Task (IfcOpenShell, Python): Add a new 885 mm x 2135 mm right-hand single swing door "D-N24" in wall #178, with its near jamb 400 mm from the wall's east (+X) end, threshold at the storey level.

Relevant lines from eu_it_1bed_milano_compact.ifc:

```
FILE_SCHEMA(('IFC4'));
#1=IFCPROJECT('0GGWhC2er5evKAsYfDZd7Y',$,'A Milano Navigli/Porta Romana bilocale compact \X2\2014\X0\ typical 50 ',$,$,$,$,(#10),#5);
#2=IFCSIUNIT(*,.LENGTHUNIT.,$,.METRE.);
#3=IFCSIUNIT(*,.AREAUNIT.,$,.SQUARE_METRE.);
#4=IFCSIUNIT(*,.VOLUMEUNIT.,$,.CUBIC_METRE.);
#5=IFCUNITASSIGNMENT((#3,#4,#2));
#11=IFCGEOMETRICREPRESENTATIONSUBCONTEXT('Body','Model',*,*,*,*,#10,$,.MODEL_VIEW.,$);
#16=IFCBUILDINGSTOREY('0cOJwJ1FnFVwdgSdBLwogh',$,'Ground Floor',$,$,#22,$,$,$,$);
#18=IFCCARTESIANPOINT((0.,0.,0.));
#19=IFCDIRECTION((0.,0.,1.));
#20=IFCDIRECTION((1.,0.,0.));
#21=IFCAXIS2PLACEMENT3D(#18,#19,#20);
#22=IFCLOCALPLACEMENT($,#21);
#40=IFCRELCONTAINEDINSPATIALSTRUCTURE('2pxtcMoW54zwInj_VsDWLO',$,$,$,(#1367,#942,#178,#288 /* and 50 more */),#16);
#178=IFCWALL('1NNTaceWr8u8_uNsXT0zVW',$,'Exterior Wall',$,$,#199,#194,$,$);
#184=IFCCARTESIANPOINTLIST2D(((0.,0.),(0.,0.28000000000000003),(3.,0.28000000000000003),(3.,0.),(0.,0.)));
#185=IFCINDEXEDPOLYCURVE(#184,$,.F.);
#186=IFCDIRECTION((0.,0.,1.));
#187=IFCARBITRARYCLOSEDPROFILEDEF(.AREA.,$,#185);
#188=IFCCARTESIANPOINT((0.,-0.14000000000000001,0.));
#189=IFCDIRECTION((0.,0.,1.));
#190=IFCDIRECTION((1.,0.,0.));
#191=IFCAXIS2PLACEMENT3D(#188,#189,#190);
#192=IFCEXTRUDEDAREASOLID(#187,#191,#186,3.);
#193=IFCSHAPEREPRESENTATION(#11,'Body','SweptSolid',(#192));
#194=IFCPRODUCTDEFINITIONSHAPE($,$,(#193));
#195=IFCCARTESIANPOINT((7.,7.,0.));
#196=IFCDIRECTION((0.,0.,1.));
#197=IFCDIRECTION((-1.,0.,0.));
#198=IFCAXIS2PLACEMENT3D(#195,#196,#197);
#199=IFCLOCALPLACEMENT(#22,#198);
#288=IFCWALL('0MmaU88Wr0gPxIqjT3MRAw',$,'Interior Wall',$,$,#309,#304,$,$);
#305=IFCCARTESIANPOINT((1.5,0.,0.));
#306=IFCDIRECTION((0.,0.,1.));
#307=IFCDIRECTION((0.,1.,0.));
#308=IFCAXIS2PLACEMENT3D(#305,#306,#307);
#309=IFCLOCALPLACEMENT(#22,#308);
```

```python
import numpy as np
import ifcopenshell
import ifcopenshell.api.feature
import ifcopenshell.api.geometry
import ifcopenshell.api.root
import ifcopenshell.api.spatial
import ifcopenshell.geom
import ifcopenshell.util.element
import ifcopenshell.util.placement
import ifcopenshell.util.representation
import ifcopenshell.util.shape
import ifcopenshell.util.unit

model = ifcopenshell.open("eu_it_1bed_milano_compact.ifc")
unit_scale = ifcopenshell.util.unit.calculate_unit_scale(model)
settings = ifcopenshell.geom.settings()


def volume(element):
    """Net volume in cubic metres, openings subtracted."""
    shape = ifcopenshell.geom.create_shape(settings, element)
    return ifcopenshell.util.shape.get_volume(shape.geometry)


wall = model.by_guid("1NNTaceWr8u8_uNsXT0zVW")
storey = ifcopenshell.util.element.get_container(wall, ifc_class="IfcBuildingStorey")
context = ifcopenshell.util.representation.get_context(model, "Model", "Body", "MODEL_VIEW")
before = volume(wall)

width, height, from_end, sill = 0.885, 2.135, 0.4, 0.0  # metres

# The wall runs along its own X axis, and the end named is its -X end.
wall_shape = ifcopenshell.geom.create_shape(settings, wall)
x, y, z = ifcopenshell.util.shape.get_vertices(wall_shape.geometry).T
start = x.min() + from_end
face, thickness = float(y.min()), float(y.max() - y.min())
wall_matrix = ifcopenshell.util.placement.get_local_placement(wall.ObjectPlacement)
level = ifcopenshell.util.placement.get_local_placement(storey.ObjectPlacement)[2, 3]


def in_wall(x, y):
    """Placement at x, y metres in the wall's axes, at sill height."""
    matrix = wall_matrix.copy()
    matrix[:, 3] = wall_matrix @ np.array([x / unit_scale, y / unit_scale, 0.0, 1.0])
    matrix[2, 3] = level + sill / unit_scale
    return matrix


# Opening: a box that overshoots both wall faces by 50 mm.
opening = ifcopenshell.api.root.create_entity(model, ifc_class="IfcOpeningElement", predefined_type="OPENING")
box = ifcopenshell.api.geometry.add_wall_representation(
    model, context=context, length=width, height=height, thickness=thickness + 0.1
)
ifcopenshell.api.geometry.assign_representation(model, product=opening, representation=box)
ifcopenshell.api.geometry.edit_object_placement(model, product=opening, matrix=in_wall(start, face - 0.05), is_si=False)
ifcopenshell.api.feature.add_feature(model, feature=opening, element=wall)

door = ifcopenshell.api.root.create_entity(model, ifc_class="IfcDoor", name="D-N24", predefined_type="DOOR")
door.OverallWidth, door.OverallHeight = width / unit_scale, height / unit_scale
door.OperationType = "SINGLE_SWING_RIGHT"
body = ifcopenshell.api.geometry.add_door_representation(
    model,
    context=context,
    overall_width=door.OverallWidth,
    overall_height=door.OverallHeight,
    operation_type="SINGLE_SWING_RIGHT",
    lining_properties={"LiningDepth": thickness / unit_scale, "ThresholdDepth": thickness / unit_scale},
)
ifcopenshell.api.geometry.assign_representation(model, product=door, representation=body)
ifcopenshell.api.spatial.assign_container(model, products=[door], relating_structure=storey)
ifcopenshell.api.feature.add_filling(model, opening=opening, element=door)

# The lining spans the wall, so the door starts at the wall face.
ifcopenshell.api.geometry.edit_object_placement(model, product=door, matrix=in_wall(start, face), is_si=False)

after = volume(wall)

print(f"wall volume {before:.3f} -> {after:.3f} m3")

model.write("eu_it_1bed_milano_compact_rev.ifc")
```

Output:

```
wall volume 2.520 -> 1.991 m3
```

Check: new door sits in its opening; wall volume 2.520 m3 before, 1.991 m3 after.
